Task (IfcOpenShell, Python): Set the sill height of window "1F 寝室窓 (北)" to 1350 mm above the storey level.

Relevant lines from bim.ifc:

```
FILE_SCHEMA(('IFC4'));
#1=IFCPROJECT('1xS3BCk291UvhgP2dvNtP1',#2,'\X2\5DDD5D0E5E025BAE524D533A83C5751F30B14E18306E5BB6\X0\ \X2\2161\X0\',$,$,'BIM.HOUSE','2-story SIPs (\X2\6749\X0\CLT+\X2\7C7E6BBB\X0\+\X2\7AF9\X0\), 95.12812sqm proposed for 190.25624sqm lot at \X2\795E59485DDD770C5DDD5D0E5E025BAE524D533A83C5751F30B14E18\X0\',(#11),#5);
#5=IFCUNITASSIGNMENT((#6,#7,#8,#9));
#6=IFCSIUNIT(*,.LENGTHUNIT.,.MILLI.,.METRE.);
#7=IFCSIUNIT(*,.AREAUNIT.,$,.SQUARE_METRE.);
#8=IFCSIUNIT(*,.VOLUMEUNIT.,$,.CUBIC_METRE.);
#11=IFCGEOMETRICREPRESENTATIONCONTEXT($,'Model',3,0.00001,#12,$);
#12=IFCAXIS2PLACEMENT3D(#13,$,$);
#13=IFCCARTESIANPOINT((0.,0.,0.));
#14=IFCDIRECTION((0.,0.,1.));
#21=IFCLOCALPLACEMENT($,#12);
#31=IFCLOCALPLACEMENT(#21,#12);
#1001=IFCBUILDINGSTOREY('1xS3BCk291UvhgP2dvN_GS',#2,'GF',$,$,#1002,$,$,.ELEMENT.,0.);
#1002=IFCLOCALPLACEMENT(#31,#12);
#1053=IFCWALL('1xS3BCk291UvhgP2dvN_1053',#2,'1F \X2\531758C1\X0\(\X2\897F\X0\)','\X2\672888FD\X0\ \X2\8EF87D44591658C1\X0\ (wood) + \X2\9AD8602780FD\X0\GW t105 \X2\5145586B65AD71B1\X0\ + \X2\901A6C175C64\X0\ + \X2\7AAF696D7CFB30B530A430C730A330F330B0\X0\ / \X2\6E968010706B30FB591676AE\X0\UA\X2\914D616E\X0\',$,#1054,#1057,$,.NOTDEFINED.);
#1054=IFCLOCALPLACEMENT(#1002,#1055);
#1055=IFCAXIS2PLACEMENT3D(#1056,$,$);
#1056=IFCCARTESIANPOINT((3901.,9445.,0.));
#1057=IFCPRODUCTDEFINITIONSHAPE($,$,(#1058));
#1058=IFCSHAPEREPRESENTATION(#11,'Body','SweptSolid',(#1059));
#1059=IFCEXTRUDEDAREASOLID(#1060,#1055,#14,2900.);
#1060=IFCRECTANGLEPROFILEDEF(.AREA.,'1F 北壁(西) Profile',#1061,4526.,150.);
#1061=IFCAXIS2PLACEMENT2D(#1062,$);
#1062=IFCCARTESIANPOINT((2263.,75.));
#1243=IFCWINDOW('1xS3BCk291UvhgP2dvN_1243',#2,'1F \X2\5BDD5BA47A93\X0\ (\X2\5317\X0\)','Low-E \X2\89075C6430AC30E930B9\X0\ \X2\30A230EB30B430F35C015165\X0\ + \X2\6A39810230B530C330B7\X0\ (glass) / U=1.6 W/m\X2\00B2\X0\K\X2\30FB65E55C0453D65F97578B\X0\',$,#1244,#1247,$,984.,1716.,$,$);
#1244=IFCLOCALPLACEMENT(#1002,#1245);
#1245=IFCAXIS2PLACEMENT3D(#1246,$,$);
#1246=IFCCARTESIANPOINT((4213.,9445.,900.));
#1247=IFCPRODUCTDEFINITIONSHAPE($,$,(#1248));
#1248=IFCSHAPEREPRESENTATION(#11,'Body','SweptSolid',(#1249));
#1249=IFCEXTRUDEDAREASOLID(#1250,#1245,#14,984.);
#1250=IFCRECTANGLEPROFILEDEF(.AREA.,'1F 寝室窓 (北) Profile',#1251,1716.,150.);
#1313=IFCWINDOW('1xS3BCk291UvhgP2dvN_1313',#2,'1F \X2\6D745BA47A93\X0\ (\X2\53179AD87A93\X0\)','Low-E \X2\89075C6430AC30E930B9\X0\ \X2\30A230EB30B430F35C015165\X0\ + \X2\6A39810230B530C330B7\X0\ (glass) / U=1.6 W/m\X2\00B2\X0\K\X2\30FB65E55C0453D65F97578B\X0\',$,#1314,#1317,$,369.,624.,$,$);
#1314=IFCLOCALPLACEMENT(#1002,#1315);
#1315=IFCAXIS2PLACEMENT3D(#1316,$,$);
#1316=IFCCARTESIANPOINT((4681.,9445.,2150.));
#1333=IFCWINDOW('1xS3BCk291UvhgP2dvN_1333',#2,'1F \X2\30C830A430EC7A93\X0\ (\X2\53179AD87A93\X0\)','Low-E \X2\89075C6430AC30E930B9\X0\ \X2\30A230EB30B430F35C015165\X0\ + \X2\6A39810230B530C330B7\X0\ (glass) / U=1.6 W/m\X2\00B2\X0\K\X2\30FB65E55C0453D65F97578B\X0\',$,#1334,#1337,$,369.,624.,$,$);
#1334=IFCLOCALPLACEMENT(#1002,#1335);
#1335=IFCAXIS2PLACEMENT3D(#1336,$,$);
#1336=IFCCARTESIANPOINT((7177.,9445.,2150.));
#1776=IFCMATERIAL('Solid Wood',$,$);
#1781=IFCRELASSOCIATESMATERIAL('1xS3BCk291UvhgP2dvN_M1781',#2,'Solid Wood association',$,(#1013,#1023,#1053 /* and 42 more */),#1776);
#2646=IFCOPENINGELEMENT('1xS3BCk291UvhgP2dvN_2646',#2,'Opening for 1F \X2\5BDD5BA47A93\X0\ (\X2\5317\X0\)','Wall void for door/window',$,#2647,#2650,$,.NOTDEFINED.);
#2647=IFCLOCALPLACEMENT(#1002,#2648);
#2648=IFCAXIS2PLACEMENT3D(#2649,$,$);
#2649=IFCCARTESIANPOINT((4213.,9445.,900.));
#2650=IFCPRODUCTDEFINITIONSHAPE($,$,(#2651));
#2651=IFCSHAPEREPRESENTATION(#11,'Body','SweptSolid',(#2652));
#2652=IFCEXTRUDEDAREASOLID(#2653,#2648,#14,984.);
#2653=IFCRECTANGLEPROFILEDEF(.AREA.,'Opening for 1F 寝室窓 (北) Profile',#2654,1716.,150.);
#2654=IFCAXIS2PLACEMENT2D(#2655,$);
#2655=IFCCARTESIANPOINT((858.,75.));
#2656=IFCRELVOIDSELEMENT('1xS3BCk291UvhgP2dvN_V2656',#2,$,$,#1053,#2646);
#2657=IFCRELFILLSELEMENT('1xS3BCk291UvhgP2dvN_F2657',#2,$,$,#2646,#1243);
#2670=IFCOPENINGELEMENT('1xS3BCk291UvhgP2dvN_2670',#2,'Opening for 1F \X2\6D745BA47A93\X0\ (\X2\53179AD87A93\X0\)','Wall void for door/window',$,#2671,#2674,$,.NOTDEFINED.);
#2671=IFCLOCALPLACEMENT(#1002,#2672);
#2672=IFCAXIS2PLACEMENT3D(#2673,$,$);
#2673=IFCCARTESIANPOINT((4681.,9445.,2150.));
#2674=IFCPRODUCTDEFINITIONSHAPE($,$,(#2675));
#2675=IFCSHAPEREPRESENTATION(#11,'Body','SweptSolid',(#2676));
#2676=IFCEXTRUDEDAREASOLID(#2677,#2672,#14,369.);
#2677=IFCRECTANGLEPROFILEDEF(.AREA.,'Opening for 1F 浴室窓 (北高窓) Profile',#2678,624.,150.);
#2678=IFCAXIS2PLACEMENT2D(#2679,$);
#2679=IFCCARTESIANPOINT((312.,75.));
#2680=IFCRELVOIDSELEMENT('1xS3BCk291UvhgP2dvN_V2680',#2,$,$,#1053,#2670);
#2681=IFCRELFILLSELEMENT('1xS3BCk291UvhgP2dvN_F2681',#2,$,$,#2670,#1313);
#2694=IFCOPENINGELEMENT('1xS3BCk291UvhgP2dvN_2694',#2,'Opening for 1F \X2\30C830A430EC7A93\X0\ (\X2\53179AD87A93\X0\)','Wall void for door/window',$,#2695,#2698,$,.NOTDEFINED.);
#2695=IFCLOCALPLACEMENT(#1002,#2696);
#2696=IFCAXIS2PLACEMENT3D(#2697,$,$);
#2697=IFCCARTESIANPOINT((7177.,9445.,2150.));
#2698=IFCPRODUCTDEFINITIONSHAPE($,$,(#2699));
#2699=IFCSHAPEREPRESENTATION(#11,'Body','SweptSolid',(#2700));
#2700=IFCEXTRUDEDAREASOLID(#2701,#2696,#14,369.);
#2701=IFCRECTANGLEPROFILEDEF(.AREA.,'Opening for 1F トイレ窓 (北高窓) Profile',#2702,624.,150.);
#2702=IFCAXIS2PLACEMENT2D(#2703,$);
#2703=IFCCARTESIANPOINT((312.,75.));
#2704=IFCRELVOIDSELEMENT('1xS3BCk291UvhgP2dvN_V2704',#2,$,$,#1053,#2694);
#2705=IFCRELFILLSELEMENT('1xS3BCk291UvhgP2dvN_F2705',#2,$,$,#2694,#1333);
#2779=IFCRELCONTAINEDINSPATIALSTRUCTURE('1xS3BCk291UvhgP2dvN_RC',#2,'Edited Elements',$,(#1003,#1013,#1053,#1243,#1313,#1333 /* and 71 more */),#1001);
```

```python
import numpy as np
import ifcopenshell
import ifcopenshell.api.geometry
import ifcopenshell.geom
import ifcopenshell.util.element
import ifcopenshell.util.placement
import ifcopenshell.util.shape
import ifcopenshell.util.unit

model = ifcopenshell.open("bim.ifc")
unit_scale = ifcopenshell.util.unit.calculate_unit_scale(model)

window = model.by_id(1243)
opening = window.FillsVoids[0].RelatingOpeningElement
storey = ifcopenshell.util.element.get_container(window, ifc_class="IfcBuildingStorey")
level = ifcopenshell.util.placement.get_local_placement(storey.ObjectPlacement)[2, 3]

# The opening's origin need not be at the sill, so measure its lowest point.
shape = ifcopenshell.geom.create_shape(ifcopenshell.geom.settings(), opening)
bottom = ifcopenshell.util.shape.get_shape_bottom_elevation(shape, shape.geometry) / unit_scale
dz = level + 1.35 / unit_scale - bottom

shift = np.array([0.0, 0.0, dz])
# The window is not placed relative to its opening, so move both.
for product in (opening, window):
    matrix = ifcopenshell.util.placement.get_local_placement(product.ObjectPlacement)
    matrix[:3, 3] += shift
    ifcopenshell.api.geometry.edit_object_placement(model, product=product, matrix=matrix, is_si=False)

print(f"moved by {dz * unit_scale:+.3f} m")

model.write("bim_updated.ifc")
```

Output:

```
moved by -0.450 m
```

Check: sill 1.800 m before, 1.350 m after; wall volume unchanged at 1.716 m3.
